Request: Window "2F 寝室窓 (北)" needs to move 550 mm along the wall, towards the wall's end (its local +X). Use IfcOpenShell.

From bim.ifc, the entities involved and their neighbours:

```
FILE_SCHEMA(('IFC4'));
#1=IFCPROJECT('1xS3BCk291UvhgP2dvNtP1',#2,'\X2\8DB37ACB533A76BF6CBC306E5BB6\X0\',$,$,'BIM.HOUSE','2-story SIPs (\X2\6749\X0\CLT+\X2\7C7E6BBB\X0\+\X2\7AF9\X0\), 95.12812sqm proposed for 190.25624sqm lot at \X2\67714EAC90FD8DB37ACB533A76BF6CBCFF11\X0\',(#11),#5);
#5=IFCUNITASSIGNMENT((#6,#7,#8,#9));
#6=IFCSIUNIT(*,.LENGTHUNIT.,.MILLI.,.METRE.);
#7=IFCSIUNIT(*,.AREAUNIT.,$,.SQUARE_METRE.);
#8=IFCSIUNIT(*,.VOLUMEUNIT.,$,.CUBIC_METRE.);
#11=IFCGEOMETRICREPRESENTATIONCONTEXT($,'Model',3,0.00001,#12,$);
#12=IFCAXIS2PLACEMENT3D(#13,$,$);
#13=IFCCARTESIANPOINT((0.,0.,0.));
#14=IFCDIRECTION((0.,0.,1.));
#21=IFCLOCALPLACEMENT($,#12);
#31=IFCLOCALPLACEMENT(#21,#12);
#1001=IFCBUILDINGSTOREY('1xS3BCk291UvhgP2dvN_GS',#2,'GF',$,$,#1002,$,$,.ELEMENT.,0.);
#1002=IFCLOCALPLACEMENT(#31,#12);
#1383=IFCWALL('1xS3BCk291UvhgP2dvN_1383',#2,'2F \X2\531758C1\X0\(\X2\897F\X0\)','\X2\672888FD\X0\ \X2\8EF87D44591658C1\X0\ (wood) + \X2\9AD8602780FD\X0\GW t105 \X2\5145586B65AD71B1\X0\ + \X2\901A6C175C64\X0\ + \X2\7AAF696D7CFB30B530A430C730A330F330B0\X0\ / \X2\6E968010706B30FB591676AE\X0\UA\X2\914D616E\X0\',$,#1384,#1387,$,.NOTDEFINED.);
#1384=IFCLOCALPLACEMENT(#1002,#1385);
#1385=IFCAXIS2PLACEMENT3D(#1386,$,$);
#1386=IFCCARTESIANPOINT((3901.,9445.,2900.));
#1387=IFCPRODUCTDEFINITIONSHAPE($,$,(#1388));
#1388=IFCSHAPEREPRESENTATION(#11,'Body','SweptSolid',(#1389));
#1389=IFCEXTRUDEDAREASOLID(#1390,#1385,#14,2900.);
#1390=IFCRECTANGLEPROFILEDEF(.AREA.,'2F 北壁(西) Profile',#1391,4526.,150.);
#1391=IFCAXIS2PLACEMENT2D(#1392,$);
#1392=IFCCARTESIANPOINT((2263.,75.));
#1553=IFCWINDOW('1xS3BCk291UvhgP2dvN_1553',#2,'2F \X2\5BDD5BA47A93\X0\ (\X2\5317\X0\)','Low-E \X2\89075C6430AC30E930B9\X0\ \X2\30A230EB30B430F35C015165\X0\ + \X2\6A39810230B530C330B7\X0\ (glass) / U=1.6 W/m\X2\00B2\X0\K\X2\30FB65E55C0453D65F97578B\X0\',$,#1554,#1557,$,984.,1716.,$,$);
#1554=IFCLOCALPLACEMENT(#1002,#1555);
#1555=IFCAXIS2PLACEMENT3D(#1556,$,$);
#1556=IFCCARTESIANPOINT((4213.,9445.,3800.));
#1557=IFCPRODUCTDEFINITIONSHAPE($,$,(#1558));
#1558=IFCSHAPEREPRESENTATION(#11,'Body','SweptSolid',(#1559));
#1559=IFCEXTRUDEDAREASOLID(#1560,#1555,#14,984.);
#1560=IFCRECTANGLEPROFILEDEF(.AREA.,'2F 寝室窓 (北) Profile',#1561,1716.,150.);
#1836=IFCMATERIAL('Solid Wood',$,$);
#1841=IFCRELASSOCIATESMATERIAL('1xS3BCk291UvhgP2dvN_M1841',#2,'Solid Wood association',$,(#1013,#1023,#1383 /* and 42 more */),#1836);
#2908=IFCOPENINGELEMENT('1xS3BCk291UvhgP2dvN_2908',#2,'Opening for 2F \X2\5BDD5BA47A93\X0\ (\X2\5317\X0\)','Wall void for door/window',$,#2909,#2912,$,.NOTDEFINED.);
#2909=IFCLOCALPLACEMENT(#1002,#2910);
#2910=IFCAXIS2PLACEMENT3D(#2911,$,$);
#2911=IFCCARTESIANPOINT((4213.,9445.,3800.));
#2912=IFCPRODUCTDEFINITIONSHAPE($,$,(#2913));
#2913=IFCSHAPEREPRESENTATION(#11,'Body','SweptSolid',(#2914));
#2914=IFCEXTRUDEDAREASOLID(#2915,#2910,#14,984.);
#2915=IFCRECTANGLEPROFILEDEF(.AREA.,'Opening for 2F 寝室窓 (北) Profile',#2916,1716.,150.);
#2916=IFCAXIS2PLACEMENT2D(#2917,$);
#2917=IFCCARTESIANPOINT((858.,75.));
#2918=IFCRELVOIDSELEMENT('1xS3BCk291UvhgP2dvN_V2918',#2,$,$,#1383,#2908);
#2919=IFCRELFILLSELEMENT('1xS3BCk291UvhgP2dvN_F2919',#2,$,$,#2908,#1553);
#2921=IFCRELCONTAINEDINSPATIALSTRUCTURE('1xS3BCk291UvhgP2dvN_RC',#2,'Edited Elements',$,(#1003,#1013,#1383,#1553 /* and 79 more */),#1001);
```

```python
import ifcopenshell
import ifcopenshell.api.geometry
import ifcopenshell.util.placement

model = ifcopenshell.open("bim.ifc")

window = model.by_id(1553)
opening = window.FillsVoids[0].RelatingOpeningElement
wall = opening.VoidsElements[0].RelatingBuildingElement

wall_matrix = ifcopenshell.util.placement.get_local_placement(wall.ObjectPlacement)
shift = wall_matrix[:3, 0] * 550.0
before = ifcopenshell.util.placement.get_local_placement(window.ObjectPlacement)[:3, 3].copy()

# The window is not placed relative to its opening, so move both.
for product in (opening, window):
    matrix = ifcopenshell.util.placement.get_local_placement(product.ObjectPlacement)
    matrix[:3, 3] += shift
    ifcopenshell.api.geometry.edit_object_placement(model, product=product, matrix=matrix, is_si=False)

after = ifcopenshell.util.placement.get_local_placement(window.ObjectPlacement)[:3, 3]
print("window moved by", (after - before).round(3) + 0.0)

model.write("bim_rev.ifc")
```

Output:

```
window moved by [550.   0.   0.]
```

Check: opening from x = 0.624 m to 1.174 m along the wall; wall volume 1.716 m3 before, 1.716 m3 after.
